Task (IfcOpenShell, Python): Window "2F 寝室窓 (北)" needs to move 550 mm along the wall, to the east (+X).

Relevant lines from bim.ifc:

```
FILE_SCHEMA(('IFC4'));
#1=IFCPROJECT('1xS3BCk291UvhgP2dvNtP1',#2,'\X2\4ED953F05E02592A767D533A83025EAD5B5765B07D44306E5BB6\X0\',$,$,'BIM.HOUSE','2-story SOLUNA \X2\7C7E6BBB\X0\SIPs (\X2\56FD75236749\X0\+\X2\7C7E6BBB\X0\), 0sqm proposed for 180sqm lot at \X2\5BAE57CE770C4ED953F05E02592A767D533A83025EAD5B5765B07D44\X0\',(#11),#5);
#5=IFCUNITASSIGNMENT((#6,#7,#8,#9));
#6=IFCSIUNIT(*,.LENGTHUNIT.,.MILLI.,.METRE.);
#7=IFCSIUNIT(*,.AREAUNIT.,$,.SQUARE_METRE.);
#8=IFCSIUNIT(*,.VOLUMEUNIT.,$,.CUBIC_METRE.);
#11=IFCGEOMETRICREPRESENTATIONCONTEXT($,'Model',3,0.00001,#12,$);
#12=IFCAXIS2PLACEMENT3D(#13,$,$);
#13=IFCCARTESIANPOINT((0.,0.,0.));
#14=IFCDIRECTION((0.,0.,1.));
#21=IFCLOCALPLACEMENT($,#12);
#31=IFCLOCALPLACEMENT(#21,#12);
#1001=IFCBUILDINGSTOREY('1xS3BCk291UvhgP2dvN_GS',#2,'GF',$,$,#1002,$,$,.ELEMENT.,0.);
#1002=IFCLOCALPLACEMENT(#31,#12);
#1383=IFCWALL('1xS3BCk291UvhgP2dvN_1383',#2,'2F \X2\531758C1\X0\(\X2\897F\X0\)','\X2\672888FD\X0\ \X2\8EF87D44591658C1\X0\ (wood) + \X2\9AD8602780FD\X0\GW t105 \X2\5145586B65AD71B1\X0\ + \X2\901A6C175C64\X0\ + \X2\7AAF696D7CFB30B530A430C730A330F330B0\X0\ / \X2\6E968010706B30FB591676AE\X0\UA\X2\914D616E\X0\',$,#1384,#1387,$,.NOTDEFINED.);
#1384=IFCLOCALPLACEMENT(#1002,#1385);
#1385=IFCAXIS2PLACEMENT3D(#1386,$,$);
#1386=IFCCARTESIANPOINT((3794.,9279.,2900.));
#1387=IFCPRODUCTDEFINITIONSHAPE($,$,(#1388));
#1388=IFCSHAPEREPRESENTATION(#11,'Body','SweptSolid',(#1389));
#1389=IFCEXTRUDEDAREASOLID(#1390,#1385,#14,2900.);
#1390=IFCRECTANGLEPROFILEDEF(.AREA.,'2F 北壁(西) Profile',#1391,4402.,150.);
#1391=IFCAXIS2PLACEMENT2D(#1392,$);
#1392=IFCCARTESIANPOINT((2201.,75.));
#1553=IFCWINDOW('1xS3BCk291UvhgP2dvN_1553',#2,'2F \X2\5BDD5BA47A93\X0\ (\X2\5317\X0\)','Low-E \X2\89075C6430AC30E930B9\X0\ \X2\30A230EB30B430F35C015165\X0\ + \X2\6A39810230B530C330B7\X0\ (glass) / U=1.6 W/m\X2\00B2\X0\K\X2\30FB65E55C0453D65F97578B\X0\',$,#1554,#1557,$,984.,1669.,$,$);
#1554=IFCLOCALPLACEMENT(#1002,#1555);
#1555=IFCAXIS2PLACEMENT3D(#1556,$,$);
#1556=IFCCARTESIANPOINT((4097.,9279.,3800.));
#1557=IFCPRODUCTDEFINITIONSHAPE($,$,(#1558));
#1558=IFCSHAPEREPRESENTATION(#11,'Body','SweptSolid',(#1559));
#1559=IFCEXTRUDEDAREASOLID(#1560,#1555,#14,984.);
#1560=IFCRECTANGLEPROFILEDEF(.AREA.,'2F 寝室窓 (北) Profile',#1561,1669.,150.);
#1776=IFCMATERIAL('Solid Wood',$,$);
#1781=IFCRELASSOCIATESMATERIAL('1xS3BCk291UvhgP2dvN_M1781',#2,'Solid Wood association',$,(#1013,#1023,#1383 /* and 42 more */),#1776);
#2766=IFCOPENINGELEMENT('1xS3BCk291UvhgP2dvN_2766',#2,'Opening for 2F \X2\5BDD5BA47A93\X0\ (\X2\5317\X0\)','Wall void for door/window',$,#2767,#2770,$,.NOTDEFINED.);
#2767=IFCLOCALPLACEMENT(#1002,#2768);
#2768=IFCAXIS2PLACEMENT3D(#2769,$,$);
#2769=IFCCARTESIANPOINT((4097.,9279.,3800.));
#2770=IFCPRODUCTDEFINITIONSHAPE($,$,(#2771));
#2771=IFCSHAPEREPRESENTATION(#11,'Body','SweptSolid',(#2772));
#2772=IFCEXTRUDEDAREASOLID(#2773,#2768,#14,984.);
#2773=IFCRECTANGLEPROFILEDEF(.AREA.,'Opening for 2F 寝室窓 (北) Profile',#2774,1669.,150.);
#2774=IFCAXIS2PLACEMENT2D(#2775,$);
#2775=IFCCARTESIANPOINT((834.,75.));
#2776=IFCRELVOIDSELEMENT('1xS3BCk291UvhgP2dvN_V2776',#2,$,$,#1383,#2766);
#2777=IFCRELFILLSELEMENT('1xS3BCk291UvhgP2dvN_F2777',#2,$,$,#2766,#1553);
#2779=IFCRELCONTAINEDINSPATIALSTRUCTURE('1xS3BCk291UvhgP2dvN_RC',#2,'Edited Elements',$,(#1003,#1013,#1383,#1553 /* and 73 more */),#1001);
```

```python
import ifcopenshell
import ifcopenshell.api.geometry
import ifcopenshell.util.placement
import ifcopenshell.util.unit

model = ifcopenshell.open("bim.ifc")
unit_scale = ifcopenshell.util.unit.calculate_unit_scale(model)

window = model.by_id(1553)
opening = window.FillsVoids[0].RelatingOpeningElement
wall = opening.VoidsElements[0].RelatingBuildingElement

wall_matrix = ifcopenshell.util.placement.get_local_placement(wall.ObjectPlacement)
shift = wall_matrix[:3, 0] * 0.55 / unit_scale
before = ifcopenshell.util.placement.get_local_placement(window.ObjectPlacement)[:3, 3].copy()

# The window is not placed relative to its opening, so move both.
for product in (opening, window):
    matrix = ifcopenshell.util.placement.get_local_placement(product.ObjectPlacement)
    matrix[:3, 3] += shift
    ifcopenshell.api.geometry.edit_object_placement(model, product=product, matrix=matrix, is_si=False)

after = ifcopenshell.util.placement.get_local_placement(window.ObjectPlacement)[:3, 3]
print("window moved by", (after - before).round(3) + 0.0)

model.write("bim_rev.ifc")
```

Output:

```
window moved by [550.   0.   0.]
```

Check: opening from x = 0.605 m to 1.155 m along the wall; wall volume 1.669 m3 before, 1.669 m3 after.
